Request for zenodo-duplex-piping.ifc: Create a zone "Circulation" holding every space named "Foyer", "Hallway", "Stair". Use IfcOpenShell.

First a look at what the model holds.

```python
import ifcopenshell

model = ifcopenshell.open("zenodo-duplex-piping.ifc")
print(model.schema)
seen = {}
for space in model.by_type("IfcSpace"):
    seen[space.LongName] = seen.get(space.LongName, 0) + 1
for name, count in sorted(seen.items(), key=str):
    print(count, "x", name)
print("zones:", [z.Name for z in model.by_type("IfcZone")][:20])
```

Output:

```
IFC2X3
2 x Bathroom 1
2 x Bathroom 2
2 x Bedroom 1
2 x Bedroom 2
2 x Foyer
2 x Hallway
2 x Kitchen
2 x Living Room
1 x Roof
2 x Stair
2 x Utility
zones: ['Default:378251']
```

```python
import ifcopenshell
import ifcopenshell.api.group
import ifcopenshell.api.root

model = ifcopenshell.open("zenodo-duplex-piping.ifc")

names = {"Foyer", "Hallway", "Stair"}
spaces = [s for s in model.by_type("IfcSpace") if s.LongName in names]

zone = ifcopenshell.api.root.create_entity(model, ifc_class="IfcZone", name="Circulation")
ifcopenshell.api.group.assign_group(model, products=spaces, group=zone)
print(len(spaces), "spaces in", zone.Name)

model.write("zenodo-duplex-piping_edited.ifc")
```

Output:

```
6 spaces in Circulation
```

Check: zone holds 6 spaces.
